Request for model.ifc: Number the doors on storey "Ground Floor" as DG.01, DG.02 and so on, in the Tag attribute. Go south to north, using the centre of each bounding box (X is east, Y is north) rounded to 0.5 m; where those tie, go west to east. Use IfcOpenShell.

First a look at what the model holds.

```python
import ifcopenshell
import ifcopenshell.util.element
import ifcopenshell.util.placement

model = ifcopenshell.open("model.ifc")
print(model.schema)
storey = next(s for s in model.by_type("IfcBuildingStorey") if s.Name == "Ground Floor")
doors = [e for e in ifcopenshell.util.element.get_decomposition(storey) if e.is_a("IfcDoor")]
for e in sorted(doors, key=lambda e: e.id()):
    origin = ifcopenshell.util.placement.get_local_placement(e.ObjectPlacement)[:3, 3]
    print(e.id(), e.Tag, e.Name, origin.round(2) + 0.0, sep=" | ")
```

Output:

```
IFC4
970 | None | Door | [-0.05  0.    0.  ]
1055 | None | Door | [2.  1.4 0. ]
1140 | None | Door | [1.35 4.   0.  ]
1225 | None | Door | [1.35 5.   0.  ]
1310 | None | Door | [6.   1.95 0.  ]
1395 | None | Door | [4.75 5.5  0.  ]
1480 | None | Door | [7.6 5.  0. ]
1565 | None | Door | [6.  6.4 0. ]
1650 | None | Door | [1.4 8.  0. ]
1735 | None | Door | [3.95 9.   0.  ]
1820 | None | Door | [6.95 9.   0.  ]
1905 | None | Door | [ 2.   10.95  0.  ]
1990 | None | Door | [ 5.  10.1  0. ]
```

```python
import ifcopenshell
import ifcopenshell.geom
import ifcopenshell.util.element
import ifcopenshell.util.shape

model = ifcopenshell.open("model.ifc")
settings = ifcopenshell.geom.settings()
settings.set("use-world-coords", True)


def centre(element):
    shape = ifcopenshell.geom.create_shape(settings, element)
    return ifcopenshell.util.shape.get_bbox_centroid(shape.geometry)


storey = next(s for s in model.by_type("IfcBuildingStorey") if s.Name == "Ground Floor")
doors = [e for e in ifcopenshell.util.element.get_decomposition(storey) if e.is_a("IfcDoor")]

# Insertion points can sit at a corner or the storey origin, so sort by the geometry (in metres).
centres = {e: centre(e) for e in doors}
doors.sort(key=lambda e: (round(centres[e][1] / 0.5), centres[e][0]))

for i, e in enumerate(doors, start=1):
    number = f"DG.{i:02d}"
    e.Tag = number
    print(e.id(), number)

model.write("model_v2.ifc")
```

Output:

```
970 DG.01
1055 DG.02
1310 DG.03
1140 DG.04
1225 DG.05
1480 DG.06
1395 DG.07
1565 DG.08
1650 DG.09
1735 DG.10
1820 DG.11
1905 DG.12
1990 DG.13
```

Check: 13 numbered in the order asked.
